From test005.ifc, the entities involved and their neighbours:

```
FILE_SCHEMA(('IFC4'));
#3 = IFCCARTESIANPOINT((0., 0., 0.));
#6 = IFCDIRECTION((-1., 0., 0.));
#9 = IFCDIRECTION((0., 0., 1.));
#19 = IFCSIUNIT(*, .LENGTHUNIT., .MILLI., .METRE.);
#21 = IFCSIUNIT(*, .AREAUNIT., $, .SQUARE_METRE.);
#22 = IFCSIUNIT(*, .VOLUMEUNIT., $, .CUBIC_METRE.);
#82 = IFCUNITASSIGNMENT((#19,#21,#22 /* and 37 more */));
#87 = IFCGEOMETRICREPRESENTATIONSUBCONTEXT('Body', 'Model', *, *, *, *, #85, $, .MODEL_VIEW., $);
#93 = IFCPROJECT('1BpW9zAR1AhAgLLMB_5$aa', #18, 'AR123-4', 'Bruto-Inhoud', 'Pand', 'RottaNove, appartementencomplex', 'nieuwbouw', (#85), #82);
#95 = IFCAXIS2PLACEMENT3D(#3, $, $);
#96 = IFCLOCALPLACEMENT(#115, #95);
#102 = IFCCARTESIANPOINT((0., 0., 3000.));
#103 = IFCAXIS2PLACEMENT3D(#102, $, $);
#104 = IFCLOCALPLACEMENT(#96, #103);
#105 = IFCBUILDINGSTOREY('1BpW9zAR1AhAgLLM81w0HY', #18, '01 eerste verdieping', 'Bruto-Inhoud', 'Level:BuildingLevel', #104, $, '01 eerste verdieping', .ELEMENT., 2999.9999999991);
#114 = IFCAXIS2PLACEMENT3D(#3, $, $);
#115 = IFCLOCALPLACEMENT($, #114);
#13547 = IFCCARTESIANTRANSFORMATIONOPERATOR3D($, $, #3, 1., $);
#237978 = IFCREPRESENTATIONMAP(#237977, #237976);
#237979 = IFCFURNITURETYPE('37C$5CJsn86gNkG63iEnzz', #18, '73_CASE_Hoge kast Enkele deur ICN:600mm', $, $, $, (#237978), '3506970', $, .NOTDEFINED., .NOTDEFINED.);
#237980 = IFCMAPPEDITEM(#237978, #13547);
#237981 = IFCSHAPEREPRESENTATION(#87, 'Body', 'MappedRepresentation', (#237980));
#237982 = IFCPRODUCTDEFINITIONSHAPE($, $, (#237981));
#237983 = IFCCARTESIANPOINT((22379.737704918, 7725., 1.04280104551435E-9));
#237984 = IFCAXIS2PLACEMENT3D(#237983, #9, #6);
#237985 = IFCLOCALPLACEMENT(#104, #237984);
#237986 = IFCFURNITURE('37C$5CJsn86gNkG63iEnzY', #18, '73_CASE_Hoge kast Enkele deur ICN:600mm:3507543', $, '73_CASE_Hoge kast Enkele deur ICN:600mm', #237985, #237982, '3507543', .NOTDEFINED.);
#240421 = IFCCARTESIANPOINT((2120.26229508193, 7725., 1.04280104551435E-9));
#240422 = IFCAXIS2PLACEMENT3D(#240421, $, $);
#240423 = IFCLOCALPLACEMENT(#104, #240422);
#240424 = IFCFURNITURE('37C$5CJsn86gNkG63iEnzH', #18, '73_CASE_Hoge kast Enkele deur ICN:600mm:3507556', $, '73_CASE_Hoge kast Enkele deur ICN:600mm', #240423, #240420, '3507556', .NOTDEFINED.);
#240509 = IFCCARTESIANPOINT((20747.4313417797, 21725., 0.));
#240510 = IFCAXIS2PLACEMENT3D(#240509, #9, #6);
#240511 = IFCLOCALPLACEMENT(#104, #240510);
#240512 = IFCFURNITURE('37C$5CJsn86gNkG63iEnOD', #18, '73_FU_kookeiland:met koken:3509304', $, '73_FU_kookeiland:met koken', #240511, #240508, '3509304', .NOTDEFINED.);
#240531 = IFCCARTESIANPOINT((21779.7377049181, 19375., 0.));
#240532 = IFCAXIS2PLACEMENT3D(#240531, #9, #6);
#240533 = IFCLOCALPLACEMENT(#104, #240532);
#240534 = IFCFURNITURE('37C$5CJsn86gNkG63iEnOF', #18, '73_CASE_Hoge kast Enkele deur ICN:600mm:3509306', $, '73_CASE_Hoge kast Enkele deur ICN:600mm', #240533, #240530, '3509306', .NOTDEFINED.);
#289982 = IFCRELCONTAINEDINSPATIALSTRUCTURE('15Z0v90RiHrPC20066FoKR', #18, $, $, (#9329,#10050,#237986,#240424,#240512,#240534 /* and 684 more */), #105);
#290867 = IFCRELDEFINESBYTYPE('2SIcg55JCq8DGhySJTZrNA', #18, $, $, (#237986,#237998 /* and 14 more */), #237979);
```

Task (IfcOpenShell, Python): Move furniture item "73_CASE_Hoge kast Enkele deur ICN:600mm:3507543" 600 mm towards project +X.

```python
import ifcopenshell
import ifcopenshell.api.geometry
import ifcopenshell.util.placement

model = ifcopenshell.open("test005.ifc")

item = model.by_guid("37C$5CJsn86gNkG63iEnzY")
matrix = ifcopenshell.util.placement.get_local_placement(item.ObjectPlacement)
matrix[0, 3] += 600.0
ifcopenshell.api.geometry.edit_object_placement(model, product=item, matrix=matrix, is_si=False)

print(ifcopenshell.util.placement.get_local_placement(item.ObjectPlacement).round(3) + 0.0)

model.write("test005_edited.ifc")
```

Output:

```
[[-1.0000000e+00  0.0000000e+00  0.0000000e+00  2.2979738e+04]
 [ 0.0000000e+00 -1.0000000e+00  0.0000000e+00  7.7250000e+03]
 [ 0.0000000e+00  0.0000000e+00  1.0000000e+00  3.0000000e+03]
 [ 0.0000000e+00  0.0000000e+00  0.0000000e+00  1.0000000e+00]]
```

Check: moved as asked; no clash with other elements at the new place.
